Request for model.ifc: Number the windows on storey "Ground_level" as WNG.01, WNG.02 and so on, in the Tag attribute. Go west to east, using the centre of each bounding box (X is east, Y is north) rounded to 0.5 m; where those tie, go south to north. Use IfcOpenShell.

First a look at what the model holds.

```python
import ifcopenshell
import ifcopenshell.util.element
import ifcopenshell.util.placement

model = ifcopenshell.open("model.ifc")
print(model.schema)
storey = next(s for s in model.by_type("IfcBuildingStorey") if s.Name == "Ground_level")
windows = [e for e in ifcopenshell.util.element.get_decomposition(storey) if e.is_a("IfcWindow")]
for e in sorted(windows, key=lambda e: e.id()):
    origin = ifcopenshell.util.placement.get_local_placement(e.ObjectPlacement)[:3, 3]
    print(e.id(), e.Tag, e.Name, origin.round(2) + 0.0, sep=" | ")
```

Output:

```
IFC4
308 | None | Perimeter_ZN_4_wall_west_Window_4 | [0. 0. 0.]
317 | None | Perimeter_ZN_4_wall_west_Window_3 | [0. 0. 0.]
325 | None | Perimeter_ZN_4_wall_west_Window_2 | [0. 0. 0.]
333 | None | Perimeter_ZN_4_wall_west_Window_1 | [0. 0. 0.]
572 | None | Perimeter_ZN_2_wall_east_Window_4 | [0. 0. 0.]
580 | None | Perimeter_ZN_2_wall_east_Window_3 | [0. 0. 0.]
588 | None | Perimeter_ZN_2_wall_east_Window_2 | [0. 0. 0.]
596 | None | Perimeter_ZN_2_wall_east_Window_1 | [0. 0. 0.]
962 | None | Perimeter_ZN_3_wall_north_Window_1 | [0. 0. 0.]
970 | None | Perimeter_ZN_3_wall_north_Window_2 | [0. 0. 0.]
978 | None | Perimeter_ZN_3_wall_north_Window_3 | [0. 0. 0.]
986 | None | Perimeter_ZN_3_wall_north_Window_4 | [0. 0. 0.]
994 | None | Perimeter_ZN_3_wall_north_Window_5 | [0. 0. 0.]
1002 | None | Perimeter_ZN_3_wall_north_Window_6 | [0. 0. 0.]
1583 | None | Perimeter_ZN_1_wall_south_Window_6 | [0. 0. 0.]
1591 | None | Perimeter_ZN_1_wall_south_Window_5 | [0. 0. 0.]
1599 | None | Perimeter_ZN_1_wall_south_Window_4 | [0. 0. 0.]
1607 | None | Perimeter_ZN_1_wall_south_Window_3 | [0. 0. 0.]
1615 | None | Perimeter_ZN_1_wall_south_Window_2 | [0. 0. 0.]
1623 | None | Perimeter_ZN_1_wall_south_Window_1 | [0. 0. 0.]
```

```python
import ifcopenshell
import ifcopenshell.geom
import ifcopenshell.util.element
import ifcopenshell.util.shape

model = ifcopenshell.open("model.ifc")
settings = ifcopenshell.geom.settings()
settings.set("use-world-coords", True)


def centre(element):
    shape = ifcopenshell.geom.create_shape(settings, element)
    return ifcopenshell.util.shape.get_bbox_centroid(shape.geometry)


storey = next(s for s in model.by_type("IfcBuildingStorey") if s.Name == "Ground_level")
windows = [e for e in ifcopenshell.util.element.get_decomposition(storey) if e.is_a("IfcWindow")]

# Insertion points can sit at a corner or the storey origin, so sort by the geometry (in metres).
centres = {e: centre(e) for e in windows}
windows.sort(key=lambda e: (round(centres[e][0] / 0.5), centres[e][1]))

for i, e in enumerate(windows, start=1):
    number = f"WNG.{i:02d}"
    e.Tag = number
    print(e.id(), number)

model.write("model_edited.ifc")
```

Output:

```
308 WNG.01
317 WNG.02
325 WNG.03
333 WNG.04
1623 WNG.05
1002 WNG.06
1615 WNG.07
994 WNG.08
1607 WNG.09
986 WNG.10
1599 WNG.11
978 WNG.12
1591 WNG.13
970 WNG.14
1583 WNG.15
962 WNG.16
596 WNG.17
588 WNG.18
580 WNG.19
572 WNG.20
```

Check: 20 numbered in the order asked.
